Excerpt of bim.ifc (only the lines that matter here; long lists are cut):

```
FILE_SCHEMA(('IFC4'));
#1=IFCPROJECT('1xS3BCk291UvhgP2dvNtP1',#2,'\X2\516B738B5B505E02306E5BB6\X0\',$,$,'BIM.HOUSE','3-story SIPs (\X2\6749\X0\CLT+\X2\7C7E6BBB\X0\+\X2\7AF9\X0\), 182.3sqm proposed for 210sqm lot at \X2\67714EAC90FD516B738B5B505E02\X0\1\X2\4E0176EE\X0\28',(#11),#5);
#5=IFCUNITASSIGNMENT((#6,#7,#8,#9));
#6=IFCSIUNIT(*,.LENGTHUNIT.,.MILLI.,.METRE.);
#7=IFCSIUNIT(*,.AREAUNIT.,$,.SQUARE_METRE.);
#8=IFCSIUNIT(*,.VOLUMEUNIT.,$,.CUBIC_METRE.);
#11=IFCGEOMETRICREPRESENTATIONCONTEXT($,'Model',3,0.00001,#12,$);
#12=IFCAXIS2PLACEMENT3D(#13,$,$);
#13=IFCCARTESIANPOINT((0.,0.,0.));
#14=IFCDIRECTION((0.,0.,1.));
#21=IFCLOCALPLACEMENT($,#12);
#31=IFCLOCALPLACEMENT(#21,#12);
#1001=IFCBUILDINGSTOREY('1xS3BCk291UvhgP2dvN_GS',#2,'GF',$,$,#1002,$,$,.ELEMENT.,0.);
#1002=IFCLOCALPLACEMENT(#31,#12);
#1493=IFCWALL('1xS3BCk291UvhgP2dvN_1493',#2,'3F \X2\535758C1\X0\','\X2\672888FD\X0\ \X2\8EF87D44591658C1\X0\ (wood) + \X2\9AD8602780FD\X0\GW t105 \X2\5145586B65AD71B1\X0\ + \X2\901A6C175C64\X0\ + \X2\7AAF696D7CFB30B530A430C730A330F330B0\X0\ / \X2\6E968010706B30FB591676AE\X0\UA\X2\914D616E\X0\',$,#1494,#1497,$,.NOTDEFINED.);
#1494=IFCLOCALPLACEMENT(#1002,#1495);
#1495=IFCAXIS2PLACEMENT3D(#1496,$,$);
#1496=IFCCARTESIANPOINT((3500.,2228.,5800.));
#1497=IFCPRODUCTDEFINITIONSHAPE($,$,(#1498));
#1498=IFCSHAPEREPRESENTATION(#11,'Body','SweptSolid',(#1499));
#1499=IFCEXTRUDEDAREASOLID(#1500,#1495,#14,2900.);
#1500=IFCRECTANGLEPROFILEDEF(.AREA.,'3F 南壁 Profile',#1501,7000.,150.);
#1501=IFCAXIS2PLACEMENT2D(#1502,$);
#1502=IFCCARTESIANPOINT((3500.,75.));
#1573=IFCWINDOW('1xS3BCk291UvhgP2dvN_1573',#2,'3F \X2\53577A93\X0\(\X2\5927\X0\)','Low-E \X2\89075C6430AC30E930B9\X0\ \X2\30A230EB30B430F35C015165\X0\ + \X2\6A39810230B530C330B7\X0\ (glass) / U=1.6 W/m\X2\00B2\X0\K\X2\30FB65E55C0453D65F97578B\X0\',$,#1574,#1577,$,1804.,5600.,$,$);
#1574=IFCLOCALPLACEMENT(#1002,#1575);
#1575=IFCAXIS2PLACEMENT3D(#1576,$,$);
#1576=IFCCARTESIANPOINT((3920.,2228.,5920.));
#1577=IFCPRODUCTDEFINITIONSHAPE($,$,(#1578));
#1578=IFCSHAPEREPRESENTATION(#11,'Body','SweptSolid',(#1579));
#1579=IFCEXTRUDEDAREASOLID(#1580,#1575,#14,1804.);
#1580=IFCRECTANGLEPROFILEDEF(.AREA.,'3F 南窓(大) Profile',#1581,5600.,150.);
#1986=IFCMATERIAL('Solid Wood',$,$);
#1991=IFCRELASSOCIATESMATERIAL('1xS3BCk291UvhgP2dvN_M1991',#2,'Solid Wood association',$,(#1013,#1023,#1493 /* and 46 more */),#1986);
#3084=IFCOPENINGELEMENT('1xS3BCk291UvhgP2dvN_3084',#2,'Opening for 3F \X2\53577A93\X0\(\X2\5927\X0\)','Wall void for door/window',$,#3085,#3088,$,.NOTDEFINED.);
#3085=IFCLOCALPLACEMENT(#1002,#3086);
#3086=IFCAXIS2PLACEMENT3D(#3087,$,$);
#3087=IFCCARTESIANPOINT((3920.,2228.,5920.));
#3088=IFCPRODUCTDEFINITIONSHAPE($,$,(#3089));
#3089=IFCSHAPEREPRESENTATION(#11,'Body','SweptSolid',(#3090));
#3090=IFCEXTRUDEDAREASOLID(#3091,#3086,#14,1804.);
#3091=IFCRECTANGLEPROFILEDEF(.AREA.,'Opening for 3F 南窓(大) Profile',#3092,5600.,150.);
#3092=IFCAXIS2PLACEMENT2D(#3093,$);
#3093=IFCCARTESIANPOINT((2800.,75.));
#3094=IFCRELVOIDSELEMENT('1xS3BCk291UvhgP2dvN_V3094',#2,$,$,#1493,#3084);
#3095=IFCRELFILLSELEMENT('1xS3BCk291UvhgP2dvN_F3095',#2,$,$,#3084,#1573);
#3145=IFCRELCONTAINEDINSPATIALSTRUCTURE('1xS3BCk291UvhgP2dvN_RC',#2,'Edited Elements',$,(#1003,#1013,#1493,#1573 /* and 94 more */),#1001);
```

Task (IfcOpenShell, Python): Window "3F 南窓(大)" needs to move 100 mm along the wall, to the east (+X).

```python
import ifcopenshell
import ifcopenshell.api.geometry
import ifcopenshell.util.placement
import ifcopenshell.util.unit

model = ifcopenshell.open("bim.ifc")
unit_scale = ifcopenshell.util.unit.calculate_unit_scale(model)

window = model.by_guid("1xS3BCk291UvhgP2dvN_1573")
opening = window.FillsVoids[0].RelatingOpeningElement
wall = opening.VoidsElements[0].RelatingBuildingElement

wall_matrix = ifcopenshell.util.placement.get_local_placement(wall.ObjectPlacement)
shift = wall_matrix[:3, 0] * 0.1 / unit_scale
before = ifcopenshell.util.placement.get_local_placement(window.ObjectPlacement)[:3, 3].copy()

# The window is not placed relative to its opening, so move both.
for product in (opening, window):
    matrix = ifcopenshell.util.placement.get_local_placement(product.ObjectPlacement)
    matrix[:3, 3] += shift
    ifcopenshell.api.geometry.edit_object_placement(model, product=product, matrix=matrix, is_si=False)

after = ifcopenshell.util.placement.get_local_placement(window.ObjectPlacement)[:3, 3]
print("window moved by", (after - before).round(3) + 0.0)

model.write("bim_v2.ifc")
```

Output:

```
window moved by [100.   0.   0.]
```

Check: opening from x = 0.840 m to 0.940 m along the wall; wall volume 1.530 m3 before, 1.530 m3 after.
